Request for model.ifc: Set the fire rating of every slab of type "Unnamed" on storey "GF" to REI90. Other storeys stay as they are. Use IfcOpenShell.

First a look at what the model holds.

```python
import ifcopenshell
import ifcopenshell.util.element

model = ifcopenshell.open("model.ifc")
print(model.schema)
storey = next(s for s in model.by_type("IfcBuildingStorey") if s.Name == "GF")
slabs = [e for e in ifcopenshell.util.element.get_decomposition(storey) if e.is_a("IfcSlab")]
seen = {}
for e in slabs:
    element_type = ifcopenshell.util.element.get_type(e)
    key = (element_type.Name if element_type != e and element_type else None, ifcopenshell.util.element.get_pset(e, "Pset_SlabCommon", "FireRating"))
    seen[key] = seen.get(key, 0) + 1
for (name, value), count in sorted(seen.items(), key=str):
    print(count, "x", name, "|", value)
```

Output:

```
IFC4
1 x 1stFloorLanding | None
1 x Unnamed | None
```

```python
import ifcopenshell
import ifcopenshell.api.pset
import ifcopenshell.util.element

model = ifcopenshell.open("model.ifc")

storey = next(s for s in model.by_type("IfcBuildingStorey") if s.Name == "GF")
slabs = [e for e in ifcopenshell.util.element.get_decomposition(storey) if e.is_a("IfcSlab")]

count = 0
for e in slabs:
    element_type = ifcopenshell.util.element.get_type(e)
    if element_type in (None, e) or element_type.Name != "Unnamed":
        continue
    # add_pset returns the element's existing set when there is one.
    pset = ifcopenshell.api.pset.add_pset(model, product=e, name="Pset_SlabCommon")
    ifcopenshell.api.pset.edit_pset(model, pset=pset, properties={"FireRating": "REI90"})
    count += 1

print(count, "slabs updated")

model.write("model-out.ifc")
```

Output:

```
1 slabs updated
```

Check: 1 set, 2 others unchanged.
